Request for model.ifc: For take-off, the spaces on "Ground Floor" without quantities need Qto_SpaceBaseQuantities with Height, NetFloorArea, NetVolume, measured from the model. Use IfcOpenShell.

First a look at what the model holds.

```python
import ifcopenshell
import ifcopenshell.util.element
import ifcopenshell.util.unit

model = ifcopenshell.open("model.ifc")
print(model.schema)
for unit_type in ("LENGTHUNIT", "AREAUNIT", "VOLUMEUNIT"):
    print(unit_type, ifcopenshell.util.unit.calculate_unit_scale(model, unit_type))
storey = next(s for s in model.by_type("IfcBuildingStorey") if s.Name == "Ground Floor")
spaces = [e for e in ifcopenshell.util.element.get_decomposition(storey) if e.is_a("IfcSpace")]
for e in sorted(spaces, key=lambda e: e.id()):
    print(e.id(), e.is_a(), e.Name, list(ifcopenshell.util.element.get_psets(e, qtos_only=True)), sep=" | ")
```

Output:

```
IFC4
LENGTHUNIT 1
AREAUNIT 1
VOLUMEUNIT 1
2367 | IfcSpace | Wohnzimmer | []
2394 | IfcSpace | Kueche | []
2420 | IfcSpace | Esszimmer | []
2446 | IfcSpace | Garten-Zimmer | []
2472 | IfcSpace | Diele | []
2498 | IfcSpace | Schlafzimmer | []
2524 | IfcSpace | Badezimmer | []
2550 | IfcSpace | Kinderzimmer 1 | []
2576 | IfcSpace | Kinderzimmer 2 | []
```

```python
import ifcopenshell
import ifcopenshell.api.pset
import ifcopenshell.geom
import ifcopenshell.util.element
import ifcopenshell.util.shape
import ifcopenshell.util.unit

model = ifcopenshell.open("model.ifc")
unit_scale = ifcopenshell.util.unit.calculate_unit_scale(model)
area_scale = ifcopenshell.util.unit.calculate_unit_scale(model, "AREAUNIT")
volume_scale = ifcopenshell.util.unit.calculate_unit_scale(model, "VOLUMEUNIT")
settings = ifcopenshell.geom.settings()

storey = next(s for s in model.by_type("IfcBuildingStorey") if s.Name == "Ground Floor")
spaces = [e for e in ifcopenshell.util.element.get_decomposition(storey) if e.is_a("IfcSpace")]

for e in sorted(spaces, key=lambda e: e.id()):
    if ifcopenshell.util.element.get_psets(e, qtos_only=True, should_inherit=False):
        continue
    # Geometry comes back in metres, in the element's own axes.
    shape = ifcopenshell.geom.create_shape(settings, e)
    values = {
        "Height": ifcopenshell.util.shape.get_z(shape.geometry) / unit_scale,
        "NetFloorArea": ifcopenshell.util.shape.get_footprint_area(shape.geometry) / area_scale,
        "NetVolume": ifcopenshell.util.shape.get_volume(shape.geometry) / volume_scale,
    }
    qto = ifcopenshell.api.pset.add_qto(model, product=e, name="Qto_SpaceBaseQuantities")
    ifcopenshell.api.pset.edit_qto(model, qto=qto, properties=values)
    print(e.id(), {k: round(v, 3) for k, v in values.items()})

model.write("model-out.ifc")
```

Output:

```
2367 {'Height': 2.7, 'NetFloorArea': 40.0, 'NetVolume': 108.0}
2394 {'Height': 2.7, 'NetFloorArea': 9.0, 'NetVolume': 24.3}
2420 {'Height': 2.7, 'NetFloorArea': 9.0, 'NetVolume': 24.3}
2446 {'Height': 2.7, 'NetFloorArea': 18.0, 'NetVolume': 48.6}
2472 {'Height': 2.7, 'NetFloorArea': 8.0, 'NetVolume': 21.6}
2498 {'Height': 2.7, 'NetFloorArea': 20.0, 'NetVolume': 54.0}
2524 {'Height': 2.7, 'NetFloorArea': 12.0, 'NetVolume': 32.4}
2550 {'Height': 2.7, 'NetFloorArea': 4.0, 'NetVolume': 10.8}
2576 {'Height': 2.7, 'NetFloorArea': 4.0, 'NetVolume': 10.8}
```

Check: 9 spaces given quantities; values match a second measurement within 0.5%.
